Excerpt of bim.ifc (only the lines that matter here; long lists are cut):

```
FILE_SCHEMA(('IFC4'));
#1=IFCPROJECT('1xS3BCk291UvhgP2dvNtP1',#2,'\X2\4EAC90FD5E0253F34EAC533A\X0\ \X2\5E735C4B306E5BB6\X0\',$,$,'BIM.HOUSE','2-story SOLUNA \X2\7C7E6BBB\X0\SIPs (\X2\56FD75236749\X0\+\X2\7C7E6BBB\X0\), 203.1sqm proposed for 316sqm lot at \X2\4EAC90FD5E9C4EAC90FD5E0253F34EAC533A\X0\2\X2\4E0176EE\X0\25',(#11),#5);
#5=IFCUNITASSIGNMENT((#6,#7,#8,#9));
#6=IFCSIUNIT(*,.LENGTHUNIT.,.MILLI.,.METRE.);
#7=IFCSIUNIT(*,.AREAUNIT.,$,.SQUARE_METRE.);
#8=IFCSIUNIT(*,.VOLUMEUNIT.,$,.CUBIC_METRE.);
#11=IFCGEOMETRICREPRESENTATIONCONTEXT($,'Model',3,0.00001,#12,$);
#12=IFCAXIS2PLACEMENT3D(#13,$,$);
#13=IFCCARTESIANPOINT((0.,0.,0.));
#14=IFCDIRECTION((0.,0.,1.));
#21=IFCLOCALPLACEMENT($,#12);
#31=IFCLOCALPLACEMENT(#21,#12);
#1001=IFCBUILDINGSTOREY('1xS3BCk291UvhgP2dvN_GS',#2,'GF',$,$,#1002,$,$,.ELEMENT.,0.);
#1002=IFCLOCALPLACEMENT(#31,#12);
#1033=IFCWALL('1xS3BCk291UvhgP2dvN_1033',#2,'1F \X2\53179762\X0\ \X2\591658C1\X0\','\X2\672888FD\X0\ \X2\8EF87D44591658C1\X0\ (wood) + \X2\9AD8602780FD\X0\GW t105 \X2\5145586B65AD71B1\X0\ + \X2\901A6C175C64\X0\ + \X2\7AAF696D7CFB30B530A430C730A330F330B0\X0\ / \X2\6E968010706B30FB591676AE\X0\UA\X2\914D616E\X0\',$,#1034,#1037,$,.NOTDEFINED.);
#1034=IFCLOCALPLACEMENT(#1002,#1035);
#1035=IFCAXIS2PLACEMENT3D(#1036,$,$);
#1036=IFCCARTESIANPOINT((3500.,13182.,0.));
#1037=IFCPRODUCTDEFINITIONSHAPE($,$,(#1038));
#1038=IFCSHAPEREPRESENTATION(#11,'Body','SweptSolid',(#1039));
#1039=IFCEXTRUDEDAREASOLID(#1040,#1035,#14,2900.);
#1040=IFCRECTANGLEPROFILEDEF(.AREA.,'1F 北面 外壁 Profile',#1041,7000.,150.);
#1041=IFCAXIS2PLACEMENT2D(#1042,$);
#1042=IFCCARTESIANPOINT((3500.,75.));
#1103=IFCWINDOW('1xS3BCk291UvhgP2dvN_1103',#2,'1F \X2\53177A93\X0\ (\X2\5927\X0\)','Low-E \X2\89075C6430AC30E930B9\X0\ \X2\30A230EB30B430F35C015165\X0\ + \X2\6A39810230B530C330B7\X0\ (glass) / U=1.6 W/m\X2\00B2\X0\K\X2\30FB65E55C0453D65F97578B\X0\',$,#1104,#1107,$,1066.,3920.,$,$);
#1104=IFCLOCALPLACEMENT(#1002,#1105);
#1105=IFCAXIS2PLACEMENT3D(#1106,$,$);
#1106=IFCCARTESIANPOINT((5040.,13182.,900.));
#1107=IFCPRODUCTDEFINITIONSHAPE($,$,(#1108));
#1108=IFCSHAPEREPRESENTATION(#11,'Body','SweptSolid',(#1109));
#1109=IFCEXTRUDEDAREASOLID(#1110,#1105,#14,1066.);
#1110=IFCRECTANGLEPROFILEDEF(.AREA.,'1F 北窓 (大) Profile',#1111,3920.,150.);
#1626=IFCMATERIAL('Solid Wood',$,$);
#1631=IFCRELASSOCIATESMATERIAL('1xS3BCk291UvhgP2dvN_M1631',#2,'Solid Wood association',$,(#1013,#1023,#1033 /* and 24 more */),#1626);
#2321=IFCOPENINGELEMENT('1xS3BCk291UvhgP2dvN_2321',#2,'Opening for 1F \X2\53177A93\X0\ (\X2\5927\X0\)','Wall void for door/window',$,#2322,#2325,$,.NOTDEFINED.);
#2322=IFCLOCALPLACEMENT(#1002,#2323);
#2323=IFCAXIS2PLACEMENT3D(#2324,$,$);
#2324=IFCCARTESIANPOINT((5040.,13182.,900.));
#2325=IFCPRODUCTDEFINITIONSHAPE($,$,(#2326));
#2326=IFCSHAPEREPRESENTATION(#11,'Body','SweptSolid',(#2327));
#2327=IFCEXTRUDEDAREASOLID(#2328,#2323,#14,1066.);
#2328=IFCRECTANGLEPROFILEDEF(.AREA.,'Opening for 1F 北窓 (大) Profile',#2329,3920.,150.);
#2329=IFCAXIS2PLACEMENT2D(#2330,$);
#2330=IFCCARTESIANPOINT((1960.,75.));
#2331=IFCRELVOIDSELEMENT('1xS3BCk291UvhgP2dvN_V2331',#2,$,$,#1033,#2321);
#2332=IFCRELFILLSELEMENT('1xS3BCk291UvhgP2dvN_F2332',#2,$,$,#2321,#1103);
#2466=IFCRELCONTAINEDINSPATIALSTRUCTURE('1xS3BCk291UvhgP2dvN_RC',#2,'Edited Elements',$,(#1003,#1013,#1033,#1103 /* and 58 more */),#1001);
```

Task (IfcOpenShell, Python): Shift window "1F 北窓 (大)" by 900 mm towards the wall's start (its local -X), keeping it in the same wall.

```python
import ifcopenshell
import ifcopenshell.api.geometry
import ifcopenshell.util.placement

model = ifcopenshell.open("bim.ifc")

window = model.by_id(1103)
opening = window.FillsVoids[0].RelatingOpeningElement
wall = opening.VoidsElements[0].RelatingBuildingElement

wall_matrix = ifcopenshell.util.placement.get_local_placement(wall.ObjectPlacement)
shift = wall_matrix[:3, 0] * -900.0
before = ifcopenshell.util.placement.get_local_placement(window.ObjectPlacement)[:3, 3].copy()

# The window is not placed relative to its opening, so move both.
for product in (opening, window):
    matrix = ifcopenshell.util.placement.get_local_placement(product.ObjectPlacement)
    matrix[:3, 3] += shift
    ifcopenshell.api.geometry.edit_object_placement(model, product=product, matrix=matrix, is_si=False)

after = ifcopenshell.util.placement.get_local_placement(window.ObjectPlacement)[:3, 3]
print("window moved by", (after - before).round(3) + 0.0)

model.write("bim_v2.ifc")
```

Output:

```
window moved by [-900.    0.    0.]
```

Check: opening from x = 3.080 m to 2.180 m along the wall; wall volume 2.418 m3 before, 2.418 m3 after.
